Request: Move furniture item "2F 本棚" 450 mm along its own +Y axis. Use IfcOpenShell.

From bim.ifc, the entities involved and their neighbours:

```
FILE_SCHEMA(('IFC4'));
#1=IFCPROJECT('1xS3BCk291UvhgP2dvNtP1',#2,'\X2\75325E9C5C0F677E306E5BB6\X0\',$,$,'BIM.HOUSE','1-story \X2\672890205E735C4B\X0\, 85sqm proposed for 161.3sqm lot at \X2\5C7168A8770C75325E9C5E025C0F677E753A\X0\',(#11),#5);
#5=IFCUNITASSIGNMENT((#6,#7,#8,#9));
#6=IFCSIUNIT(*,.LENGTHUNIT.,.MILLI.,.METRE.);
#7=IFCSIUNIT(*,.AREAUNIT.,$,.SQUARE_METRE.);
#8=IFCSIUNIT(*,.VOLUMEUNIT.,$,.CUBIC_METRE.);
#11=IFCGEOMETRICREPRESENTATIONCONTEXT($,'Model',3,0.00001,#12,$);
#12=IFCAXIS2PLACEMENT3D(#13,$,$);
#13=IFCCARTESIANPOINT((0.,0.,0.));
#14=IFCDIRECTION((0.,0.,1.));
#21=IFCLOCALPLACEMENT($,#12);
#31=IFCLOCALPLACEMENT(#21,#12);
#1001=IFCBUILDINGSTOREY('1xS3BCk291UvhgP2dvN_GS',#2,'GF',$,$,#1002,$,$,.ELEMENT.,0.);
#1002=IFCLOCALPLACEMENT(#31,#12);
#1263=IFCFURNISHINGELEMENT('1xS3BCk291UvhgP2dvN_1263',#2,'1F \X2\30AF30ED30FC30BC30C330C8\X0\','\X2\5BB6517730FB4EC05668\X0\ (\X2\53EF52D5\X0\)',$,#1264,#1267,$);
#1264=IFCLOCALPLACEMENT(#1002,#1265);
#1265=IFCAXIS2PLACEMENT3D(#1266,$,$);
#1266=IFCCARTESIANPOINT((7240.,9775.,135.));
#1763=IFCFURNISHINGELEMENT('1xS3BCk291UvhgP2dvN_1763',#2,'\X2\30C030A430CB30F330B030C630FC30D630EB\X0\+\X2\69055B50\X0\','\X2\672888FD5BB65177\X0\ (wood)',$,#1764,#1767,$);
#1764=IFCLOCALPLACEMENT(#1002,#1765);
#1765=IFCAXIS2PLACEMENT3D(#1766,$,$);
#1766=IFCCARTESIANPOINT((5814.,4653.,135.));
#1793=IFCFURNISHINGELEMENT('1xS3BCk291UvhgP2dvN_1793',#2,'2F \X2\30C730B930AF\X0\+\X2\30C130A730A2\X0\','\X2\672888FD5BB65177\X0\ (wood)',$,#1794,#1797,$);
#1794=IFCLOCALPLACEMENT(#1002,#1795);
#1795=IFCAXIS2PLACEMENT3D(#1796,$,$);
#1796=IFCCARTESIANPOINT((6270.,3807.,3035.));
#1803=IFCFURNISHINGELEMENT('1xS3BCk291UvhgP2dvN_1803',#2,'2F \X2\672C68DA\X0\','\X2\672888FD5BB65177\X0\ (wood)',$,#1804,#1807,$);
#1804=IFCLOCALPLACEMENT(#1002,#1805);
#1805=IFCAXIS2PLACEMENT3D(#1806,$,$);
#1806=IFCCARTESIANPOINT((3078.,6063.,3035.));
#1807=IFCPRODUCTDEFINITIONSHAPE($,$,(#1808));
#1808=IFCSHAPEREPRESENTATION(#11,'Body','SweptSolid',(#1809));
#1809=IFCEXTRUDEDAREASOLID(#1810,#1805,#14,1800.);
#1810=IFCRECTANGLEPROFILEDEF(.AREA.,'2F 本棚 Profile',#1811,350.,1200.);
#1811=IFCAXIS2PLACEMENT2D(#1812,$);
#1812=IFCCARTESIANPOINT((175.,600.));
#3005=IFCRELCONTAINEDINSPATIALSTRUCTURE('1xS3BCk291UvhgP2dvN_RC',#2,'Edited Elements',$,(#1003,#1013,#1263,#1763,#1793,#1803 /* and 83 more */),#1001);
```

```python
import ifcopenshell
import ifcopenshell.api.geometry
import ifcopenshell.util.placement

model = ifcopenshell.open("bim.ifc")

item = model.by_id(1803)
matrix = ifcopenshell.util.placement.get_local_placement(item.ObjectPlacement)
matrix[:3, 3] += matrix[:3, 1] * 450.0
ifcopenshell.api.geometry.edit_object_placement(model, product=item, matrix=matrix, is_si=False)

print(ifcopenshell.util.placement.get_local_placement(item.ObjectPlacement).round(3) + 0.0)

model.write("bim_updated.ifc")
```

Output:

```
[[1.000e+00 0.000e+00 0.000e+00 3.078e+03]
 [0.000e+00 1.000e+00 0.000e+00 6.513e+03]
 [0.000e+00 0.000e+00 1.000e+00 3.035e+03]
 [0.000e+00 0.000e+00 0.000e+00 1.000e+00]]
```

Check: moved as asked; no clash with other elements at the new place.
